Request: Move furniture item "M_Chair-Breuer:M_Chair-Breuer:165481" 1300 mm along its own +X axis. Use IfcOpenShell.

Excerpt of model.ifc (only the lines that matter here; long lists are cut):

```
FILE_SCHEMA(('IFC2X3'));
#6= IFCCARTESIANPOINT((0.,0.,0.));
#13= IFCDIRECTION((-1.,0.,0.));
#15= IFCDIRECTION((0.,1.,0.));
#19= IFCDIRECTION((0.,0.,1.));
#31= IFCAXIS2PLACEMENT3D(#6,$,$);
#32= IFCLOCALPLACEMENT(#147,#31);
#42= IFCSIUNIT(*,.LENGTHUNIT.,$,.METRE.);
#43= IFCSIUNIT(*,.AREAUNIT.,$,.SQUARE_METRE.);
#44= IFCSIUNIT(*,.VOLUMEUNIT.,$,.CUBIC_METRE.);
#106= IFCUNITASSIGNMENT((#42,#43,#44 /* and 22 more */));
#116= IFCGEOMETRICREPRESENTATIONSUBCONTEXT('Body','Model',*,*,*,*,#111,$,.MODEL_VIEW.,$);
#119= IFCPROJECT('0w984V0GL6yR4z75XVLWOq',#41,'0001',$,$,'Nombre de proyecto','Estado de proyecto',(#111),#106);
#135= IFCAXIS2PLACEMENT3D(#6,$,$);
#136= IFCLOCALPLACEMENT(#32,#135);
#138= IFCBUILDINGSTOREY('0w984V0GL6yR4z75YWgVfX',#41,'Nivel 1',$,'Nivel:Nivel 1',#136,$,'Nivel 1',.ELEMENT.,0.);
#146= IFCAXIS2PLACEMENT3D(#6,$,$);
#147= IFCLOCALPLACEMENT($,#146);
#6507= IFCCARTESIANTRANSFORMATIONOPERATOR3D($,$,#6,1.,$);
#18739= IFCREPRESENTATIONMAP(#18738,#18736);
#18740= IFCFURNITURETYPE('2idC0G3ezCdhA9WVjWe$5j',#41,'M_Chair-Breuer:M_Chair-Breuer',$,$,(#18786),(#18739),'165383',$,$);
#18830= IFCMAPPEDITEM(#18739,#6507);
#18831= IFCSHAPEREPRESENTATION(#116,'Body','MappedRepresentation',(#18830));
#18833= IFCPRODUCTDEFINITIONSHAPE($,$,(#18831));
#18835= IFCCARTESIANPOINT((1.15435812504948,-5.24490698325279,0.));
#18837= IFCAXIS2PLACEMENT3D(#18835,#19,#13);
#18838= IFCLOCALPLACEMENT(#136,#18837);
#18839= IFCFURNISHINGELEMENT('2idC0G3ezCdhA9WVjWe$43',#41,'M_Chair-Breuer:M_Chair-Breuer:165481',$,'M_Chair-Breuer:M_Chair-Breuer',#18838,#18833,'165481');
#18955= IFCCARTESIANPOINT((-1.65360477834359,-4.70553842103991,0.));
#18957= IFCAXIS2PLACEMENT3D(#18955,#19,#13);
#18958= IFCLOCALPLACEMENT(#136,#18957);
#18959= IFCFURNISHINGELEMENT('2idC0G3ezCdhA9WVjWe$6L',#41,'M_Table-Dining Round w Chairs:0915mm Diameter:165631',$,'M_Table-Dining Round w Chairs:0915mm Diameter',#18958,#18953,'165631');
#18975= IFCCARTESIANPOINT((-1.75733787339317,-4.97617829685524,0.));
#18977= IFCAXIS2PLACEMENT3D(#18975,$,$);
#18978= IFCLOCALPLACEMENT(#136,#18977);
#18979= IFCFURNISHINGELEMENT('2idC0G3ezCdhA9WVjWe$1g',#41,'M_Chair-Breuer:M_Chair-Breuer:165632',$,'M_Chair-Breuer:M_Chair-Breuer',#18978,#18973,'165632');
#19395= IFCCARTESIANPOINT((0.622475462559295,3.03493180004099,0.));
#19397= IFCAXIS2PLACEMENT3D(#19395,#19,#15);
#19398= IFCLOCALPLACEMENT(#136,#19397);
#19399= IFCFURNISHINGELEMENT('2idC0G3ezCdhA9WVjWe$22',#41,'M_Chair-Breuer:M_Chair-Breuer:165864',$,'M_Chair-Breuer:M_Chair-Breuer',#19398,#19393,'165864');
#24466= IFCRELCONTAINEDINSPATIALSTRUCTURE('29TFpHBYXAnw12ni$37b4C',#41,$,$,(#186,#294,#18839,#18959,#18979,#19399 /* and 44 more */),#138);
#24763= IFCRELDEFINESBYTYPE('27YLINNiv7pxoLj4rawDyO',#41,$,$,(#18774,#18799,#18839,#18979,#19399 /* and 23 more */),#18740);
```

```python
import ifcopenshell
import ifcopenshell.api.geometry
import ifcopenshell.util.placement
import ifcopenshell.util.unit

model = ifcopenshell.open("model.ifc")
unit_scale = ifcopenshell.util.unit.calculate_unit_scale(model)

item = model.by_guid("2idC0G3ezCdhA9WVjWe$43")
matrix = ifcopenshell.util.placement.get_local_placement(item.ObjectPlacement)
matrix[:3, 3] += matrix[:3, 0] * 1.3 / unit_scale
ifcopenshell.api.geometry.edit_object_placement(model, product=item, matrix=matrix, is_si=False)

print(ifcopenshell.util.placement.get_local_placement(item.ObjectPlacement).round(3) + 0.0)

model.write("model_updated.ifc")
```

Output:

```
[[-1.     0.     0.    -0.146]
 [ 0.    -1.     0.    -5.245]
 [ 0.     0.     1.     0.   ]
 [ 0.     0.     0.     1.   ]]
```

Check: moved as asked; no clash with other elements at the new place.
